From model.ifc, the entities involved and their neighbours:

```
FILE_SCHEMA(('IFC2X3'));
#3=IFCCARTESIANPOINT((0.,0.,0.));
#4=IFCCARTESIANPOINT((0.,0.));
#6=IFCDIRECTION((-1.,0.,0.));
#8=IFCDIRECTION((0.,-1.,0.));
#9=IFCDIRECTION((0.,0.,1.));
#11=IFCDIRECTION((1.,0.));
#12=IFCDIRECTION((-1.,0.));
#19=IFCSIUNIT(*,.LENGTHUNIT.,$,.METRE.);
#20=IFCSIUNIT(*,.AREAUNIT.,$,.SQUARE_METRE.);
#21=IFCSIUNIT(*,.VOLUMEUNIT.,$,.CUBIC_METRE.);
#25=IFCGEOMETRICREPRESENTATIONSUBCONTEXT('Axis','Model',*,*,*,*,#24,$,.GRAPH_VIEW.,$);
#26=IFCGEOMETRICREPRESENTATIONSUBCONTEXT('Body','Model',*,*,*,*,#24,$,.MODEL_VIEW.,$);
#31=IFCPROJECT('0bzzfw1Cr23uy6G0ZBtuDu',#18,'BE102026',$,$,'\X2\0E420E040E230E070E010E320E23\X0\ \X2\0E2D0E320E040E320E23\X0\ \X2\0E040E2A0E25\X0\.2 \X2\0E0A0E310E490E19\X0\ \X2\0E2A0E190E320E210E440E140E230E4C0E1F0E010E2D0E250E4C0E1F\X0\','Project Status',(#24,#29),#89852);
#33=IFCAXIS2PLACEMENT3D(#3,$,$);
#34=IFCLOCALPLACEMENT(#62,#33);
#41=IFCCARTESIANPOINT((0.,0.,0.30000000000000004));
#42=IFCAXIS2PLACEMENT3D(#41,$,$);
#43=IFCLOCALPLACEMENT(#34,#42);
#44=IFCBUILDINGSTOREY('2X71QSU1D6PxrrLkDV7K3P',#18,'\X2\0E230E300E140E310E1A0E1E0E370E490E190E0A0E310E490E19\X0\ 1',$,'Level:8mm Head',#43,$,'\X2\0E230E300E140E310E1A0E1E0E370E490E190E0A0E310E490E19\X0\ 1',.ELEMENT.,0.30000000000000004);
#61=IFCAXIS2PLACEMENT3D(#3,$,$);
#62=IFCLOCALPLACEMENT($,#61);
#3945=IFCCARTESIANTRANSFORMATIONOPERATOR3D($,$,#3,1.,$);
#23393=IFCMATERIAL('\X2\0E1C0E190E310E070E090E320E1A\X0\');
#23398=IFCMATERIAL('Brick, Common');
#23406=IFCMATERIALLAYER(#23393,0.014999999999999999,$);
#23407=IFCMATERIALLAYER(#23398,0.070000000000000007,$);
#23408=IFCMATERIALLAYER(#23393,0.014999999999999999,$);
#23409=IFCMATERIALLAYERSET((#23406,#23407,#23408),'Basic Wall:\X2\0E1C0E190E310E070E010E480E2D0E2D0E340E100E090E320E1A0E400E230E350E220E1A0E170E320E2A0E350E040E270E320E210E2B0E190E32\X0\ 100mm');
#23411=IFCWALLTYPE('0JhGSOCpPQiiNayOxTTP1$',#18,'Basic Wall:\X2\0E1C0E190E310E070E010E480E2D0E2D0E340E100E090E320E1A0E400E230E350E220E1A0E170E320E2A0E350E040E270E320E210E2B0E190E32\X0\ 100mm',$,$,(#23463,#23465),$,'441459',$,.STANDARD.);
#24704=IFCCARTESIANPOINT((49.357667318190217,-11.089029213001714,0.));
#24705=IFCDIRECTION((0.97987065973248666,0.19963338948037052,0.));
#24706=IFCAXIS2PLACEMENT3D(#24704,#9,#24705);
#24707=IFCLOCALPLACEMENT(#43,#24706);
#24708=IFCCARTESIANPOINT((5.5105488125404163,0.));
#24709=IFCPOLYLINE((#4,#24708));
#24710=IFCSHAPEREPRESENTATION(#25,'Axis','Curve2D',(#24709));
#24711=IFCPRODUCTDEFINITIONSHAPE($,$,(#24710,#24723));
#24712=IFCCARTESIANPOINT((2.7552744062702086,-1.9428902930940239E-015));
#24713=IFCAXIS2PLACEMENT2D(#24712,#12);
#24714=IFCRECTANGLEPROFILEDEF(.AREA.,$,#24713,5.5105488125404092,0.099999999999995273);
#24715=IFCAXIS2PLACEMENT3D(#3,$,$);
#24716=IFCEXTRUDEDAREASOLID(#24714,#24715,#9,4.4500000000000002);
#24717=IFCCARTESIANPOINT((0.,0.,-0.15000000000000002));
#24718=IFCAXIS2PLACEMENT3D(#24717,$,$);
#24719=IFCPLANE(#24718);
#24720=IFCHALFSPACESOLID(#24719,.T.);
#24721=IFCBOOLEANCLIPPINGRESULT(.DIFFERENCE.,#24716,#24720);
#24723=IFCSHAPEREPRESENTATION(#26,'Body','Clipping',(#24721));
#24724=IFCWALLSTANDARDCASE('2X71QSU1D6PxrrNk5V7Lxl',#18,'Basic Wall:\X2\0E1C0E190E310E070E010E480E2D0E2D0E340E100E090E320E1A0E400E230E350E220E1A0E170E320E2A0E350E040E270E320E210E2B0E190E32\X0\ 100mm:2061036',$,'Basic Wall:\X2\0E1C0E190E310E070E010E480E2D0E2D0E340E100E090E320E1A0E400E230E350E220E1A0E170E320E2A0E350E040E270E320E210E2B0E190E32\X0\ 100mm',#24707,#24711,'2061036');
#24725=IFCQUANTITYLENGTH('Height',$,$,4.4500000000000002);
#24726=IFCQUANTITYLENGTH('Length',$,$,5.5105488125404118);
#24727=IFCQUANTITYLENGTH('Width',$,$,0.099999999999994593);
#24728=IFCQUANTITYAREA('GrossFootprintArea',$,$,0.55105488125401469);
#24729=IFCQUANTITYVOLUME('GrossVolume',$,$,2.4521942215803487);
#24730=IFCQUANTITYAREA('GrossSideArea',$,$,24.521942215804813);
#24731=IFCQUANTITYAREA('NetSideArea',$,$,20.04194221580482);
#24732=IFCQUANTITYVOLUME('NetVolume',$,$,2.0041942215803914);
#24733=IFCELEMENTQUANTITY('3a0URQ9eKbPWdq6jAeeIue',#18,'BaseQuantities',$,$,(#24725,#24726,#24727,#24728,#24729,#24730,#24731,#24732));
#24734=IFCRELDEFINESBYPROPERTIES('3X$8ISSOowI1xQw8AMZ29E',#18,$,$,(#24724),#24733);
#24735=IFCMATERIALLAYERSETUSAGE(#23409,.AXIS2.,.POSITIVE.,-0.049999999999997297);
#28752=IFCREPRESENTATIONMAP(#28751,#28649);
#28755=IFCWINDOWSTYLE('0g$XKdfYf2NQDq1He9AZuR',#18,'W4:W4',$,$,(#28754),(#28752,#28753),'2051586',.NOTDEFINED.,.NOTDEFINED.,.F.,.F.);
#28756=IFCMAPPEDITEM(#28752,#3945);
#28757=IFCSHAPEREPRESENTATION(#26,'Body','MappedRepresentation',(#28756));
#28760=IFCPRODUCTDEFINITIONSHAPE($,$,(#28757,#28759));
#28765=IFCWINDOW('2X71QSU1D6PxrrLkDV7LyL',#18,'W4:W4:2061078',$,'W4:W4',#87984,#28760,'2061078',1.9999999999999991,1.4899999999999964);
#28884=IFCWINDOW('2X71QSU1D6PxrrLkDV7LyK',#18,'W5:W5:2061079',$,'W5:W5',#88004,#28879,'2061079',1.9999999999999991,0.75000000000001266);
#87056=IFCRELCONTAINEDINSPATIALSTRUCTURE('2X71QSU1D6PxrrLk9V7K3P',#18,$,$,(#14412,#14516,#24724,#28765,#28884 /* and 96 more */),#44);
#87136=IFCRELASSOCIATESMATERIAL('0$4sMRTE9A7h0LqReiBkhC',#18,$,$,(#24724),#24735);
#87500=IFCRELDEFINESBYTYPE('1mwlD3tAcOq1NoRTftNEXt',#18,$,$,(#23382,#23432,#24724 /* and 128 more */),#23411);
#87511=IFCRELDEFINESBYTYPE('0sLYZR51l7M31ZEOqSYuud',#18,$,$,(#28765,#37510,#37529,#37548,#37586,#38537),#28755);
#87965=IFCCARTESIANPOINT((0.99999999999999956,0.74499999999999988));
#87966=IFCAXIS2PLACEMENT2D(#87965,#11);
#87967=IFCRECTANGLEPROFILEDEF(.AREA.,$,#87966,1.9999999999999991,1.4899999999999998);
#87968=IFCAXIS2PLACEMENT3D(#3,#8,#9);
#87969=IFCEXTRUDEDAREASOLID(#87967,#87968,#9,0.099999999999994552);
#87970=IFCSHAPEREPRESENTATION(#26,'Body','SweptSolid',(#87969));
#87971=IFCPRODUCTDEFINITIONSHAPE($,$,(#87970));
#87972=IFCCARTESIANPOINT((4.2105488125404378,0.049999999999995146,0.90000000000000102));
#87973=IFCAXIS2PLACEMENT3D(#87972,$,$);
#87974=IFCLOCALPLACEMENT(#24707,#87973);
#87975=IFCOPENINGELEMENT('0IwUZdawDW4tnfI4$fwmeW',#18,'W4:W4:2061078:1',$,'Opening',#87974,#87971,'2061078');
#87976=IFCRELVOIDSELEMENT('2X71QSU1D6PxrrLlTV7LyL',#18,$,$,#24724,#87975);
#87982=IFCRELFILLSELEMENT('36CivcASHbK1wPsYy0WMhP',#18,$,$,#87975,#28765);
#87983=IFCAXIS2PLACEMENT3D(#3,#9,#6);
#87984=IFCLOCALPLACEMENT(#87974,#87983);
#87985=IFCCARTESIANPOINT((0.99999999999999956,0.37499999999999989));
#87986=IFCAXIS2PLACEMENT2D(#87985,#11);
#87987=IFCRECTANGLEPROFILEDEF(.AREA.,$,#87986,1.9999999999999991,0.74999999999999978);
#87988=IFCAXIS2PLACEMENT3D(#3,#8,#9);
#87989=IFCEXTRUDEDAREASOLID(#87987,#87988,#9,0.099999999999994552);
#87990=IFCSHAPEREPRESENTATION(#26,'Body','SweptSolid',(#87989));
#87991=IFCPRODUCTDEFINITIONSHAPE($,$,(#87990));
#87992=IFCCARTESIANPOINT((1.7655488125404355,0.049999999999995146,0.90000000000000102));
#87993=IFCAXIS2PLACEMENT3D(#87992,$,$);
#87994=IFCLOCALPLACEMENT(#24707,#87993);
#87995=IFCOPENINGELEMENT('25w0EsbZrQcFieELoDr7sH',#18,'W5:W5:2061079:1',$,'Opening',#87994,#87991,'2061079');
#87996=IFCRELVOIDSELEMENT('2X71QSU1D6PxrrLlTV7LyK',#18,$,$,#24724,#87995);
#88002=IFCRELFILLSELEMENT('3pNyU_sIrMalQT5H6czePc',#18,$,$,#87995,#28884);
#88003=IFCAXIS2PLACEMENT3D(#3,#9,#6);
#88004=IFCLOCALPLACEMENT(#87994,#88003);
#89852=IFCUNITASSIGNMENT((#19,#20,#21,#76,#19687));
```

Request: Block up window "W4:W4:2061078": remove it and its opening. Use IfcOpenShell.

```python
import ifcopenshell
import ifcopenshell.api.feature
import ifcopenshell.api.pset
import ifcopenshell.api.root
import ifcopenshell.geom
import ifcopenshell.util.element
import ifcopenshell.util.shape
import ifcopenshell.util.unit

model = ifcopenshell.open("model.ifc")
area_scale = ifcopenshell.util.unit.calculate_unit_scale(model, "AREAUNIT")
volume_scale = ifcopenshell.util.unit.calculate_unit_scale(model, "VOLUMEUNIT")
settings = ifcopenshell.geom.settings()


def volume(element):
    """Net volume in cubic metres, openings subtracted."""
    shape = ifcopenshell.geom.create_shape(settings, element)
    return ifcopenshell.util.shape.get_volume(shape.geometry)


window = model.by_guid("2X71QSU1D6PxrrLkDV7LyL")
opening = window.FillsVoids[0].RelatingOpeningElement
wall = opening.VoidsElements[0].RelatingBuildingElement
before = volume(wall)

ifcopenshell.api.root.remove_product(model, product=window)
ifcopenshell.api.feature.remove_feature(model, feature=opening)

after = volume(wall)
thickness = 0.1  # wall thickness in metres

# Update the wall's stored quantities.
qto = model.by_id(ifcopenshell.util.element.get_pset(wall, "BaseQuantities", should_inherit=False)["id"])
ifcopenshell.api.pset.edit_qto(model, qto=qto, properties={
    "NetSideArea": after / thickness / area_scale,
    "NetVolume": after / volume_scale,
})

print(f"wall volume {before:.3f} -> {after:.3f} m3")

model.write("model_v2.ifc")
```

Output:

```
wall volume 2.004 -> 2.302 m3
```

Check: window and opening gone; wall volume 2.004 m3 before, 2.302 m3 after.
